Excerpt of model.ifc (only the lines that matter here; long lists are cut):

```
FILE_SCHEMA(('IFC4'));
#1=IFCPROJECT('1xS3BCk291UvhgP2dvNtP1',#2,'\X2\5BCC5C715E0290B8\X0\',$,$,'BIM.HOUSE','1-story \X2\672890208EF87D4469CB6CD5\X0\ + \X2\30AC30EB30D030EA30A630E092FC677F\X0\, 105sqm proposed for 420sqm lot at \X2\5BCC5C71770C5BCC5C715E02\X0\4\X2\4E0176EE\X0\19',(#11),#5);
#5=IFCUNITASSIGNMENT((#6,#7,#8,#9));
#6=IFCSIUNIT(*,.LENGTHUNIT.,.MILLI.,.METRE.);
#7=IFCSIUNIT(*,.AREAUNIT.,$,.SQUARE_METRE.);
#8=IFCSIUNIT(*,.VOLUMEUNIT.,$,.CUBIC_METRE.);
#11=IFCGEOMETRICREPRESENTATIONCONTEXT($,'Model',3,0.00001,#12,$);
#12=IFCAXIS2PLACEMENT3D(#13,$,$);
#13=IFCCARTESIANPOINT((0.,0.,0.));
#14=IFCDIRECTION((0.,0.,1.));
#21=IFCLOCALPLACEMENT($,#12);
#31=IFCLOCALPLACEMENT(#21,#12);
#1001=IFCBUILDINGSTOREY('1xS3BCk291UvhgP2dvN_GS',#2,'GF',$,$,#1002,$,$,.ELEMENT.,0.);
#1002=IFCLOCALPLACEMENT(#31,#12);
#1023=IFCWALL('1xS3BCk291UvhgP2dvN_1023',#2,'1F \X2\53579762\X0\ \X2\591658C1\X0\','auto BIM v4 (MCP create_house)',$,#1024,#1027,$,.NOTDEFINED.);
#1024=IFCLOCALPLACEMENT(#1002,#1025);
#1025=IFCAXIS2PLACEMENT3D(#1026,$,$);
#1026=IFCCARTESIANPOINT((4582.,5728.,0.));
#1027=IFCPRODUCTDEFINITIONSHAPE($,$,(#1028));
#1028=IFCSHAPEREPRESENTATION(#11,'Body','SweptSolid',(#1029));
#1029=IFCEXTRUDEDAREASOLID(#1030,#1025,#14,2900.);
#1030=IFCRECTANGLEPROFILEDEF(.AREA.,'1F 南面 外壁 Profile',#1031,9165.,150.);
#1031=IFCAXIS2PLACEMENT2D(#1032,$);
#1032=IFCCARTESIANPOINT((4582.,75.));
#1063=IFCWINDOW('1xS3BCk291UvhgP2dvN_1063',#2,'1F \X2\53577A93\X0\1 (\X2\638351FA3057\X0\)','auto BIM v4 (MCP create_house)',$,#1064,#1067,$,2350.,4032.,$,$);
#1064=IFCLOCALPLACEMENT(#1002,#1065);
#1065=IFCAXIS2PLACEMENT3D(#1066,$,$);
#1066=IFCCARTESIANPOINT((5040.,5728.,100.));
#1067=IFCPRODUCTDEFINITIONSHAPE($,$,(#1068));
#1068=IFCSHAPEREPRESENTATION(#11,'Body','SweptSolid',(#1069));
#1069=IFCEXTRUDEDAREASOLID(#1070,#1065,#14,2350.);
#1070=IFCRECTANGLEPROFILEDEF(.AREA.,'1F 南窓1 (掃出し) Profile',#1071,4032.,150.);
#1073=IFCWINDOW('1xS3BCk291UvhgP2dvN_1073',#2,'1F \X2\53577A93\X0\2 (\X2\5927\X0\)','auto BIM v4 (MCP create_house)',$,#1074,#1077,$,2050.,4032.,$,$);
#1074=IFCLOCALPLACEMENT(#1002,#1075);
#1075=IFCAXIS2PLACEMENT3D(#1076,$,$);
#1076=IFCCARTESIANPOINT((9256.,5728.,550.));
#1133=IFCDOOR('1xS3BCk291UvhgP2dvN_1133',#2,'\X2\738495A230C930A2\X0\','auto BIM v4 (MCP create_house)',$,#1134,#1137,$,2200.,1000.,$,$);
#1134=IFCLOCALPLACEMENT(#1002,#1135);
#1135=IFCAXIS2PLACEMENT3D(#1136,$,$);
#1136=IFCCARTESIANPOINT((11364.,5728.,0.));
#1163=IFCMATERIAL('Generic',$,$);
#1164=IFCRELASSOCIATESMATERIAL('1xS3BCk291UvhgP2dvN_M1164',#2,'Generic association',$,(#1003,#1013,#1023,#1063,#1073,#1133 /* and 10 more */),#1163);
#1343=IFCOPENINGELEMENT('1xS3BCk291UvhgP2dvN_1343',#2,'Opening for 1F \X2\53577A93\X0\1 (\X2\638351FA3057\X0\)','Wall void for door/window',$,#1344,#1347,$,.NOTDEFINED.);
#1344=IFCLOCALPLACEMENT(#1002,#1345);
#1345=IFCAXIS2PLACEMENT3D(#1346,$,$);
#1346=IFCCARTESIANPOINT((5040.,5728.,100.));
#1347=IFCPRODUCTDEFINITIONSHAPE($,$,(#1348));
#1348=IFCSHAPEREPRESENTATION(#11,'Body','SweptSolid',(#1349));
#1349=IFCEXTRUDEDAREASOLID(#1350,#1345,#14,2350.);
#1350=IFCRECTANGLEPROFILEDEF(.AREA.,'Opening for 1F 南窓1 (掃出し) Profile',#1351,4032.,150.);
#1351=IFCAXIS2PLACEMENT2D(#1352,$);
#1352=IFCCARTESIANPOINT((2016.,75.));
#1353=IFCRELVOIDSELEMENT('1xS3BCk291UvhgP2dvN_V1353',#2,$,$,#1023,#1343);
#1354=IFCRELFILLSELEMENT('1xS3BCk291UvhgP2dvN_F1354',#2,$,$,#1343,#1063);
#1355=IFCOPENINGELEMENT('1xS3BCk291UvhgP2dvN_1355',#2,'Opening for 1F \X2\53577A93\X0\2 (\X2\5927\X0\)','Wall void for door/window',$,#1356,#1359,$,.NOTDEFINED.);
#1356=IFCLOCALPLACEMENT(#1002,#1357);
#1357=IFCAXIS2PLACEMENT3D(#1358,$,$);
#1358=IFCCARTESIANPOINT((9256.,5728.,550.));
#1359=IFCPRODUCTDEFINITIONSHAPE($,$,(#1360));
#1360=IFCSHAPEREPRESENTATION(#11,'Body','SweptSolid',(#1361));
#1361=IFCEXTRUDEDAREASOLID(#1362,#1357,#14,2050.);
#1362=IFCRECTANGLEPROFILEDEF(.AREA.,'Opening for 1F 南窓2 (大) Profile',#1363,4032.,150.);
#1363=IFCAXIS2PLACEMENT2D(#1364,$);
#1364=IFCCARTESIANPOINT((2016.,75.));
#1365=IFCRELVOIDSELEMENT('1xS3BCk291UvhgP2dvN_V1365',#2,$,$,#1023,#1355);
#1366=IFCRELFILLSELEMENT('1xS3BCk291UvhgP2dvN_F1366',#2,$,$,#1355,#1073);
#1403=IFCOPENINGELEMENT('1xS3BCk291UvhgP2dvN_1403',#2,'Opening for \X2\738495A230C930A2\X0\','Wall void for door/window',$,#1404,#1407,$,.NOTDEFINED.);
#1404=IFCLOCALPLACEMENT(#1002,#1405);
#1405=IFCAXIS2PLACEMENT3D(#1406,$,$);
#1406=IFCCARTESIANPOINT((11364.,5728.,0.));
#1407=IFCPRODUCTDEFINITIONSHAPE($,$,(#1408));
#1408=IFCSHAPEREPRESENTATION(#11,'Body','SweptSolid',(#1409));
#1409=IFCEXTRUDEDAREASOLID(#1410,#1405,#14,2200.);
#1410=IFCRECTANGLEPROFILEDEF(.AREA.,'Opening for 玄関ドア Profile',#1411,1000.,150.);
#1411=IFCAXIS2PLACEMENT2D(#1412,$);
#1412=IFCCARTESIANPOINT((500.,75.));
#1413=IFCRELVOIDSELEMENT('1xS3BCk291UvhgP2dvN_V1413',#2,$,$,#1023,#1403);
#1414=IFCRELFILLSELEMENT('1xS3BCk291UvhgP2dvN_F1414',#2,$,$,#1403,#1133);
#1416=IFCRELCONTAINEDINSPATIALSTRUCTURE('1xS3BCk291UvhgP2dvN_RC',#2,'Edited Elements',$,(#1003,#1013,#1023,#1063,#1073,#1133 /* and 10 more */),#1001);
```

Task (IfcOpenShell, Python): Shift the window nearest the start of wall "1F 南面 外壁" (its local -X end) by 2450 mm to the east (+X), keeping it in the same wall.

```python
import ifcopenshell
import ifcopenshell.api.geometry
import ifcopenshell.util.placement
import ifcopenshell.util.unit

model = ifcopenshell.open("model.ifc")
unit_scale = ifcopenshell.util.unit.calculate_unit_scale(model)

window = model.by_guid("1xS3BCk291UvhgP2dvN_1063")
opening = window.FillsVoids[0].RelatingOpeningElement
wall = opening.VoidsElements[0].RelatingBuildingElement

wall_matrix = ifcopenshell.util.placement.get_local_placement(wall.ObjectPlacement)
shift = wall_matrix[:3, 0] * 2.45 / unit_scale
before = ifcopenshell.util.placement.get_local_placement(window.ObjectPlacement)[:3, 3].copy()

# The window is not placed relative to its opening, so move both.
for product in (opening, window):
    matrix = ifcopenshell.util.placement.get_local_placement(product.ObjectPlacement)
    matrix[:3, 3] += shift
    ifcopenshell.api.geometry.edit_object_placement(model, product=product, matrix=matrix, is_si=False)

after = ifcopenshell.util.placement.get_local_placement(window.ObjectPlacement)[:3, 3]
print("window moved by", (after - before).round(3) + 0.0)

model.write("model_v2.ifc")
```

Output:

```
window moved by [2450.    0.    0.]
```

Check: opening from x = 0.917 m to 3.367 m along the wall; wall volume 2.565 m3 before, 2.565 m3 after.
